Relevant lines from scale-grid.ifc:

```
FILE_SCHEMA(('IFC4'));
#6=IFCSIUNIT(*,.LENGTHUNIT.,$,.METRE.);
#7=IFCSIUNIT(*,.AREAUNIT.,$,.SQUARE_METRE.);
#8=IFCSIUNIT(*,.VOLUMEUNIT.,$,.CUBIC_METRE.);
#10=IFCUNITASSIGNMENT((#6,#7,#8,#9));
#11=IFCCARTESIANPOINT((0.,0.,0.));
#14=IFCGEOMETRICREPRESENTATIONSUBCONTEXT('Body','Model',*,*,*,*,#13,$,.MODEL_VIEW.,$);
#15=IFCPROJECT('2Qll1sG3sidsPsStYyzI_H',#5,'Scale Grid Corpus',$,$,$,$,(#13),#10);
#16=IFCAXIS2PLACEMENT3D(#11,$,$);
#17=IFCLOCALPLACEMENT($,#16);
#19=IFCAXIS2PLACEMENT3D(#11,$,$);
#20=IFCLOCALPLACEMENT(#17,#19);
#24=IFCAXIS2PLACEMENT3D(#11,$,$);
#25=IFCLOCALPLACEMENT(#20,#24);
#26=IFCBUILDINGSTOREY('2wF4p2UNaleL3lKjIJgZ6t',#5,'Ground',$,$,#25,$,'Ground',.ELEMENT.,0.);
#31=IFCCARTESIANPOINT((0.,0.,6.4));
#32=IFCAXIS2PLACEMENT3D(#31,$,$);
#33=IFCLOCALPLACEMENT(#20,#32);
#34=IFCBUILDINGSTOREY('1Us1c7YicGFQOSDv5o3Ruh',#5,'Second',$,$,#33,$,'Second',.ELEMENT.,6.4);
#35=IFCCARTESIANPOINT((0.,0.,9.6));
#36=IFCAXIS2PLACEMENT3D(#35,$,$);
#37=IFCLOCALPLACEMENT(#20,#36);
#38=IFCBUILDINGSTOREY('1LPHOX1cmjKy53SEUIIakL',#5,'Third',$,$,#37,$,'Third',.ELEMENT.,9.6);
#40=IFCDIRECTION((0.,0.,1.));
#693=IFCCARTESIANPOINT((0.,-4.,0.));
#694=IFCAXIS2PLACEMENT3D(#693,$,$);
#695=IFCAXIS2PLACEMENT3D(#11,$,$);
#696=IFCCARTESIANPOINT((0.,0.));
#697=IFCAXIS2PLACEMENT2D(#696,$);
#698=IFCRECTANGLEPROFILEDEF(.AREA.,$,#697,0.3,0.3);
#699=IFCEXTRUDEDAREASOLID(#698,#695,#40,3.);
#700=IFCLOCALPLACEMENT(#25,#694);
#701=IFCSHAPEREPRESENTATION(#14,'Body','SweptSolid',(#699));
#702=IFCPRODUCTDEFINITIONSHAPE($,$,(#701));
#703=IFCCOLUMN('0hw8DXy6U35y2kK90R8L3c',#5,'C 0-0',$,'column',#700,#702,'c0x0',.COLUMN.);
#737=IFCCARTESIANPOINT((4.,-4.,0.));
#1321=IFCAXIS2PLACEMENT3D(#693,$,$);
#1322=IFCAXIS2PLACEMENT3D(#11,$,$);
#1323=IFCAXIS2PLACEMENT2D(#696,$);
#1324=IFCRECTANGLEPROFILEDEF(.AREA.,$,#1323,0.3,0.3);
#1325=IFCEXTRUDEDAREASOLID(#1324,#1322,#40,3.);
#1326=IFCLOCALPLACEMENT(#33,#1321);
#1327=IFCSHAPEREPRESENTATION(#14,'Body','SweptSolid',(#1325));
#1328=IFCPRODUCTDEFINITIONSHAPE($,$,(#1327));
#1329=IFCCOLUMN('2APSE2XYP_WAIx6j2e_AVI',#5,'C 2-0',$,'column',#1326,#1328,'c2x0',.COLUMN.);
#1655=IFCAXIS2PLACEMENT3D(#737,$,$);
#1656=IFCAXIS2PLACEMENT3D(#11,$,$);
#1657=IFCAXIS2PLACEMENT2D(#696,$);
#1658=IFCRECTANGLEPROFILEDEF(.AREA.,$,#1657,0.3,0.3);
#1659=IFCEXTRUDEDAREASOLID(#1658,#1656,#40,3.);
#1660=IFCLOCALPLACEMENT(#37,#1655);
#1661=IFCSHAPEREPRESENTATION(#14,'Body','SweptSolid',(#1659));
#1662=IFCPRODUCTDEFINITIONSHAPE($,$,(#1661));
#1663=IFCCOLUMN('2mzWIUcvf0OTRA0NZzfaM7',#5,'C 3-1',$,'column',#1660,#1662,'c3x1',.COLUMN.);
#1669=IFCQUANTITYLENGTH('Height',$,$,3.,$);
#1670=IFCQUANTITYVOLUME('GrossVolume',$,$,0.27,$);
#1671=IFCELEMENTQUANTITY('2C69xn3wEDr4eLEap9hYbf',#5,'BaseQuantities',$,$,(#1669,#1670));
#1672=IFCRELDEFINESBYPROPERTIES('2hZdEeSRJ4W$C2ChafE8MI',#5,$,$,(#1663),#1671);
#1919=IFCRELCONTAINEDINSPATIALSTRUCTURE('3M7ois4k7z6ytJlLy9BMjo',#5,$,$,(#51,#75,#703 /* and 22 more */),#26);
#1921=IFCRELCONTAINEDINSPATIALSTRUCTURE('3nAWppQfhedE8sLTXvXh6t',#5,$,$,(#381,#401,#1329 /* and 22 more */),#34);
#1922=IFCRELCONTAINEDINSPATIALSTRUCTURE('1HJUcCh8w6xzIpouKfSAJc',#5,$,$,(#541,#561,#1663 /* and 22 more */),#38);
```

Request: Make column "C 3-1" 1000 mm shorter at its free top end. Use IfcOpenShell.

```python
import ifcopenshell
import ifcopenshell.api.pset
import ifcopenshell.util.element
import ifcopenshell.util.representation
import ifcopenshell.util.unit

model = ifcopenshell.open("scale-grid.ifc")
unit_scale = ifcopenshell.util.unit.calculate_unit_scale(model)

member = model.by_guid("2mzWIUcvf0OTRA0NZzfaM7")
change = -1 / unit_scale

# The extrusion runs towards the end named, so only its depth changes.
body = ifcopenshell.util.representation.get_representation(member, "Model", "Body")
solid = body.Items[0]
old_length = solid.Depth
solid.Depth += change

# Update the stored length and volume.
qto = model.by_id(ifcopenshell.util.element.get_pset(member, "BaseQuantities", should_inherit=False)["id"])
ifcopenshell.api.pset.edit_qto(model, qto=qto, properties={
    "Height": solid.Depth,
    "GrossVolume": ifcopenshell.util.element.get_pset(member, "BaseQuantities", "GrossVolume") * solid.Depth / old_length,
})

print(f"length {old_length:g} -> {solid.Depth:g}")

model.write("scale-grid-out.ifc")
```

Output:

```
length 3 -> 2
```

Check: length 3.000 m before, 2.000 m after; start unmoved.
